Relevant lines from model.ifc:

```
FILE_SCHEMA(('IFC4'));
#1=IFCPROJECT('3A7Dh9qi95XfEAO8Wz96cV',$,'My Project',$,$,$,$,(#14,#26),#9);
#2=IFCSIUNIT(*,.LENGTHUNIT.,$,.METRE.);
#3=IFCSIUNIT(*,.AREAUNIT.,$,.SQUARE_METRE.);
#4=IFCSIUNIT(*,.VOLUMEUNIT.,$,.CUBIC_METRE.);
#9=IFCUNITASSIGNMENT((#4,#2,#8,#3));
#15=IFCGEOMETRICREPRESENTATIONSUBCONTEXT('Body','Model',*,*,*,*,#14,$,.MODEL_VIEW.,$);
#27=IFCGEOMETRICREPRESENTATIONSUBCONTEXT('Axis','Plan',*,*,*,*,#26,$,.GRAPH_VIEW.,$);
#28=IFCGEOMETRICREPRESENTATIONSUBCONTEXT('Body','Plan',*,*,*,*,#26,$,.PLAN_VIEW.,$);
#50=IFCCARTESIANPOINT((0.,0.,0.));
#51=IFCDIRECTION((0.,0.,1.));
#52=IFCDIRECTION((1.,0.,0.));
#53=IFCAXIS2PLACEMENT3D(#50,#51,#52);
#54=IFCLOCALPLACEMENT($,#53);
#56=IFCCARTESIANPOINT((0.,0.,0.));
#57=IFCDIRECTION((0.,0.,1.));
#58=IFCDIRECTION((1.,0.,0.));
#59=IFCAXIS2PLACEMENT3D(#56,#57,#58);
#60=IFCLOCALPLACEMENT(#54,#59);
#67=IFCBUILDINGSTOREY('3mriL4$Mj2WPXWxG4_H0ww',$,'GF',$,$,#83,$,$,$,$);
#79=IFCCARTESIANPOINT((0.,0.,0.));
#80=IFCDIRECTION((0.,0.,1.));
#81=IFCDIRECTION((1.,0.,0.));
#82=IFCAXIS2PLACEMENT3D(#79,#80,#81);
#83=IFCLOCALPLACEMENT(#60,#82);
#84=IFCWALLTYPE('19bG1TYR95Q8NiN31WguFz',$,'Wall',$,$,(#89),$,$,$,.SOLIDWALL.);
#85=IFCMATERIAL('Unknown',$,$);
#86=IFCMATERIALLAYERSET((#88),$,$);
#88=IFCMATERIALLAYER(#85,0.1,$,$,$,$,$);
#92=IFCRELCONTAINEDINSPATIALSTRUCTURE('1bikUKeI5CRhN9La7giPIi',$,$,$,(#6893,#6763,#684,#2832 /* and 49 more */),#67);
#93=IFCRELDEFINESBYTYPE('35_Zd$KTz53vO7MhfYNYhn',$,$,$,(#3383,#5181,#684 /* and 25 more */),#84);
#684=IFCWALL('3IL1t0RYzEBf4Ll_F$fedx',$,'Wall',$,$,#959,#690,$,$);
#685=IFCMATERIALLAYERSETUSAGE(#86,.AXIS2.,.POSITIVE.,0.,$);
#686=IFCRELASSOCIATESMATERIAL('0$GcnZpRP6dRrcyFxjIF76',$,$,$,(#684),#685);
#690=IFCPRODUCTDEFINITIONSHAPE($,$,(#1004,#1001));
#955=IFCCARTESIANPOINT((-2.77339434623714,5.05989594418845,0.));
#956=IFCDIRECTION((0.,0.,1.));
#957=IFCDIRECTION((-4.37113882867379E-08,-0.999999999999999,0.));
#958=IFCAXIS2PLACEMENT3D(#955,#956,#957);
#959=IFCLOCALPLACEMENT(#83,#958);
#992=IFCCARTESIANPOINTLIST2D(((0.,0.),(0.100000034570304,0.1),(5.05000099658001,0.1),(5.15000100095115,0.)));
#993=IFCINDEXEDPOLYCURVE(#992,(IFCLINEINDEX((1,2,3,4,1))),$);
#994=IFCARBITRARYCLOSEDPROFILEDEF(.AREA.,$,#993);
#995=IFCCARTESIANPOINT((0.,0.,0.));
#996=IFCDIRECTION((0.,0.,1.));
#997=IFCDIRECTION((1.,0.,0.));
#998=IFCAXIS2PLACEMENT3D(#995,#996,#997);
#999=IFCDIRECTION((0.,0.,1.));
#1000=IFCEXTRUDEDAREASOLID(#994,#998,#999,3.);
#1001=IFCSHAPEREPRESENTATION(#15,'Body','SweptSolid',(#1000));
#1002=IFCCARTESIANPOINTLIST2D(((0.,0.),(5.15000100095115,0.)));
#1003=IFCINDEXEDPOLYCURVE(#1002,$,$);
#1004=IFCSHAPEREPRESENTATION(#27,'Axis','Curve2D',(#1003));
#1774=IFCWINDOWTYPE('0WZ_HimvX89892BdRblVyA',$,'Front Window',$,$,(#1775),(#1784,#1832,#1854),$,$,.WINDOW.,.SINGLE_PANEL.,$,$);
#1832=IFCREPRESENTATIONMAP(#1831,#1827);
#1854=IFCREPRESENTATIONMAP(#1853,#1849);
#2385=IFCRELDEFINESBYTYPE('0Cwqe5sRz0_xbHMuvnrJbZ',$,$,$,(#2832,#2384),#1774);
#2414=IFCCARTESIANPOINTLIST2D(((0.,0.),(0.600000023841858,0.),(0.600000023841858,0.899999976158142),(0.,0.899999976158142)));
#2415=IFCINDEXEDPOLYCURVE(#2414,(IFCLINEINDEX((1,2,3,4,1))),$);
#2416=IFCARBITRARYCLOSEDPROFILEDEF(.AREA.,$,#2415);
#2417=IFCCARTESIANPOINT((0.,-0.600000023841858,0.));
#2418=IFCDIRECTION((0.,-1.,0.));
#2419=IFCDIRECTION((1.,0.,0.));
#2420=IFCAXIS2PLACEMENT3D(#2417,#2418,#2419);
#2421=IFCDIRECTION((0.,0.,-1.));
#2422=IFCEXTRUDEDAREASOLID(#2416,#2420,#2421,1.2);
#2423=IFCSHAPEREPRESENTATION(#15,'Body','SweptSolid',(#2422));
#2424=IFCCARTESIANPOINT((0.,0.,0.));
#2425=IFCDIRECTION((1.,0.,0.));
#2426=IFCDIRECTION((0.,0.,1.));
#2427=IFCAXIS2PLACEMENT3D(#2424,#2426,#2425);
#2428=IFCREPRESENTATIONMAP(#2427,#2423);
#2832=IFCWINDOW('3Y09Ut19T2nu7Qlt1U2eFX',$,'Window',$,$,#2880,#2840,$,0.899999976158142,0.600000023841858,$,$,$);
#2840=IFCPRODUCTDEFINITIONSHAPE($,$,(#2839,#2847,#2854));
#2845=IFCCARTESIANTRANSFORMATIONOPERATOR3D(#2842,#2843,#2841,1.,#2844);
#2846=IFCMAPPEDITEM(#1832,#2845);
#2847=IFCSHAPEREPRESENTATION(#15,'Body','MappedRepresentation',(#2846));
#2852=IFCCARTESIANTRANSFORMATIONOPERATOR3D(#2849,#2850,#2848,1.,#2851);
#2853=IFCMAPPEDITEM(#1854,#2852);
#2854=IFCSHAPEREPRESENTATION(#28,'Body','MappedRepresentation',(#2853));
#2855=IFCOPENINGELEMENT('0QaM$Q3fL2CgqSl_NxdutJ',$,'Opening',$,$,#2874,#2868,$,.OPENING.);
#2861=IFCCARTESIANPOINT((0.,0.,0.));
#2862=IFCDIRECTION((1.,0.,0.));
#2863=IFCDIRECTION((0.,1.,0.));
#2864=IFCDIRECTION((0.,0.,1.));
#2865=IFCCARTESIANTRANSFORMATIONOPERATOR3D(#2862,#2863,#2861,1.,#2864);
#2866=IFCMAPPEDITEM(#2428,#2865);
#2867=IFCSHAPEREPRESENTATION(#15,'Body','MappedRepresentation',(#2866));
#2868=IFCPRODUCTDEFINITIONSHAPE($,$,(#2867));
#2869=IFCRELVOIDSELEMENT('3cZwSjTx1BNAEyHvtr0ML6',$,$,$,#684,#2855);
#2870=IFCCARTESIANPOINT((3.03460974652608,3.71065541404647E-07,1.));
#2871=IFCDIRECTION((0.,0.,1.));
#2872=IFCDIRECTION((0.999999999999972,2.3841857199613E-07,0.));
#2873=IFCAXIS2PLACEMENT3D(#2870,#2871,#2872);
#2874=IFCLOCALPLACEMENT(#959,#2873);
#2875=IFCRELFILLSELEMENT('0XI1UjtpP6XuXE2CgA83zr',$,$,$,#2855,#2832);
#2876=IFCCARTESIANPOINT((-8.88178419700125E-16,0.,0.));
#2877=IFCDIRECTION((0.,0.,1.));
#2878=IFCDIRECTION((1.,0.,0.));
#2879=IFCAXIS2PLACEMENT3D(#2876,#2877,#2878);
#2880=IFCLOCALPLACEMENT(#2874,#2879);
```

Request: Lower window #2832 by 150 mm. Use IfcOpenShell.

```python
import numpy as np
import ifcopenshell
import ifcopenshell.api.geometry
import ifcopenshell.util.placement
import ifcopenshell.util.unit

model = ifcopenshell.open("model.ifc")
unit_scale = ifcopenshell.util.unit.calculate_unit_scale(model)

window = model.by_guid("3Y09Ut19T2nu7Qlt1U2eFX")
opening = window.FillsVoids[0].RelatingOpeningElement
dz = -0.15 / unit_scale

shift = np.array([0.0, 0.0, dz])
# The window is placed relative to its opening, so it follows when the opening moves.
matrix = ifcopenshell.util.placement.get_local_placement(opening.ObjectPlacement)
matrix[:3, 3] += shift
ifcopenshell.api.geometry.edit_object_placement(
    model, product=opening, matrix=matrix, is_si=False, should_transform_children=True
)

print(f"moved by {dz * unit_scale:+.3f} m")

model.write("model_updated.ifc")
```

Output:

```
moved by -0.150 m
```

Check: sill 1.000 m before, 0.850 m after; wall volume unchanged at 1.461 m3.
